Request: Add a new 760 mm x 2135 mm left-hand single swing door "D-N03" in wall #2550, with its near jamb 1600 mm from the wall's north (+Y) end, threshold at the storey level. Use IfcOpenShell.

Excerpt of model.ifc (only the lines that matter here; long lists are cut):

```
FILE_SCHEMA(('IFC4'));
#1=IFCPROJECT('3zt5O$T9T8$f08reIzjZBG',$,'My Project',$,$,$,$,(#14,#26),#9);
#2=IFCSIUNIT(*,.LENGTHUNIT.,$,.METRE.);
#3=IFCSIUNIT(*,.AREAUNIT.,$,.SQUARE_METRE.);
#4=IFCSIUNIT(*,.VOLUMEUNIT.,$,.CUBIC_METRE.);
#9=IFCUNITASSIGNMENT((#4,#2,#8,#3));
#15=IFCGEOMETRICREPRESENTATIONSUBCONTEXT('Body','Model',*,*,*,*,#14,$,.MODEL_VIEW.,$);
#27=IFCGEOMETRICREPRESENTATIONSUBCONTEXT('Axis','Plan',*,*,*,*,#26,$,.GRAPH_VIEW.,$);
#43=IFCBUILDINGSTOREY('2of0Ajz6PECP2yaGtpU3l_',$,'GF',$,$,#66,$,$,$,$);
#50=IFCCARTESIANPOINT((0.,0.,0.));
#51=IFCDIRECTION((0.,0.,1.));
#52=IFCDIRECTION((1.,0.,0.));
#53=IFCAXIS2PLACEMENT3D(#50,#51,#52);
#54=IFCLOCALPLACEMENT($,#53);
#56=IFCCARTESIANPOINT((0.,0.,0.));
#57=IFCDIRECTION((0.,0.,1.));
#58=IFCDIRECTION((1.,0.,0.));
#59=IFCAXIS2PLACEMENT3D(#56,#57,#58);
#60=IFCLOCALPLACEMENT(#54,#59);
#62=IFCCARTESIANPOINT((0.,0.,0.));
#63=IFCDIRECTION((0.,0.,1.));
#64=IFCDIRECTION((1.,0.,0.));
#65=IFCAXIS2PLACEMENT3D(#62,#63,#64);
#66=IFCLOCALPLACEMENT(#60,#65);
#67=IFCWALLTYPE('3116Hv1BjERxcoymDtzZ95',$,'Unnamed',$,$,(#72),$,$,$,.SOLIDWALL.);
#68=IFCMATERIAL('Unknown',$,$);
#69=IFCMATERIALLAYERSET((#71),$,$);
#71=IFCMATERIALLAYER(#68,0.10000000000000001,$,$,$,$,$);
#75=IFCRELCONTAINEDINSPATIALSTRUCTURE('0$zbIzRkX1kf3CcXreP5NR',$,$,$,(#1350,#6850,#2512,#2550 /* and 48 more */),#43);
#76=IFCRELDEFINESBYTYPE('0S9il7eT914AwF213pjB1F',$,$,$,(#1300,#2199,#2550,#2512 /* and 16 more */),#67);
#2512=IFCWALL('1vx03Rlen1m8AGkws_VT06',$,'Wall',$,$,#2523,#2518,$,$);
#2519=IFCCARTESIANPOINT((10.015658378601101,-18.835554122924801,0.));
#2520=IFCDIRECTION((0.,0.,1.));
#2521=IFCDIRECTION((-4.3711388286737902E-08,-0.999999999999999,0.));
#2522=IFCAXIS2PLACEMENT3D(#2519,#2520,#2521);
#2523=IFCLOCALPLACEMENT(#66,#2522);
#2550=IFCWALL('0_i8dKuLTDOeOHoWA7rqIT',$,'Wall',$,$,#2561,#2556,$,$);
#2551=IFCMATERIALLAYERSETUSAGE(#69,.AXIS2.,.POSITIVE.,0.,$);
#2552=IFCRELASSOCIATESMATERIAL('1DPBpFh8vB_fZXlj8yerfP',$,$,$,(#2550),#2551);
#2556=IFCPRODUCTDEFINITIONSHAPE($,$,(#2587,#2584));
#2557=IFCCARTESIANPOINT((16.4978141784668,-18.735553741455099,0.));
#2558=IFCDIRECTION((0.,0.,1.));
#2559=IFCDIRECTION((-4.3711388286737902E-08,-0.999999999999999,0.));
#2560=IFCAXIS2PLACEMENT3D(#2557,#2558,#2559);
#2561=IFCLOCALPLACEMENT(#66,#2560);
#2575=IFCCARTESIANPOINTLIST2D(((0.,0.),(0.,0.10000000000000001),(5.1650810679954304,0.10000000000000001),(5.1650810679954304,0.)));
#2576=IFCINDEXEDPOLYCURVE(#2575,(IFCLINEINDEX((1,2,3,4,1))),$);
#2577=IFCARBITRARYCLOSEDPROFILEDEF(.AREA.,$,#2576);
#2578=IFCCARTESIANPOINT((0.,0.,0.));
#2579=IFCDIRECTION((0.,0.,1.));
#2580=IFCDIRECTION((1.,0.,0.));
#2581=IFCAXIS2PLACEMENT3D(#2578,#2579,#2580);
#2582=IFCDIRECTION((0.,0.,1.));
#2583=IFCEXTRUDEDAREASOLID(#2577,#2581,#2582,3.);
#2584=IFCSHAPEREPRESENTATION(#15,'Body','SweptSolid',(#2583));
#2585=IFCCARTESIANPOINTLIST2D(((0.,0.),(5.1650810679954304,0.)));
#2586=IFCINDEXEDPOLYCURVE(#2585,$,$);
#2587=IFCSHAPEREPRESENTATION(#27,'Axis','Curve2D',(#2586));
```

```python
import numpy as np
import ifcopenshell
import ifcopenshell.api.feature
import ifcopenshell.api.geometry
import ifcopenshell.api.root
import ifcopenshell.api.spatial
import ifcopenshell.geom
import ifcopenshell.util.element
import ifcopenshell.util.placement
import ifcopenshell.util.representation
import ifcopenshell.util.shape
import ifcopenshell.util.unit

model = ifcopenshell.open("model.ifc")
unit_scale = ifcopenshell.util.unit.calculate_unit_scale(model)
settings = ifcopenshell.geom.settings()


def volume(element):
    """Net volume in cubic metres, openings subtracted."""
    shape = ifcopenshell.geom.create_shape(settings, element)
    return ifcopenshell.util.shape.get_volume(shape.geometry)


wall = model.by_guid("0_i8dKuLTDOeOHoWA7rqIT")
storey = ifcopenshell.util.element.get_container(wall, ifc_class="IfcBuildingStorey")
context = ifcopenshell.util.representation.get_context(model, "Model", "Body", "MODEL_VIEW")
before = volume(wall)

width, height, from_end, sill = 0.76, 2.135, 1.6, 0.0  # metres

# The wall runs along its own X axis, and the end named is its -X end.
wall_shape = ifcopenshell.geom.create_shape(settings, wall)
x, y, z = ifcopenshell.util.shape.get_vertices(wall_shape.geometry).T
start = x.min() + from_end
face, thickness = float(y.min()), float(y.max() - y.min())
wall_matrix = ifcopenshell.util.placement.get_local_placement(wall.ObjectPlacement)
level = ifcopenshell.util.placement.get_local_placement(storey.ObjectPlacement)[2, 3]


def in_wall(x, y):
    """Placement at x, y metres in the wall's axes, at sill height."""
    matrix = wall_matrix.copy()
    matrix[:, 3] = wall_matrix @ np.array([x / unit_scale, y / unit_scale, 0.0, 1.0])
    matrix[2, 3] = level + sill / unit_scale
    return matrix


# Opening: a box that overshoots both wall faces by 50 mm.
opening = ifcopenshell.api.root.create_entity(model, ifc_class="IfcOpeningElement", predefined_type="OPENING")
box = ifcopenshell.api.geometry.add_wall_representation(
    model, context=context, length=width, height=height, thickness=thickness + 0.1
)
ifcopenshell.api.geometry.assign_representation(model, product=opening, representation=box)
ifcopenshell.api.geometry.edit_object_placement(model, product=opening, matrix=in_wall(start, face - 0.05), is_si=False)
ifcopenshell.api.feature.add_feature(model, feature=opening, element=wall)

door = ifcopenshell.api.root.create_entity(model, ifc_class="IfcDoor", name="D-N03", predefined_type="DOOR")
door.OverallWidth, door.OverallHeight = width / unit_scale, height / unit_scale
door.OperationType = "SINGLE_SWING_LEFT"
body = ifcopenshell.api.geometry.add_door_representation(
    model,
    context=context,
    overall_width=door.OverallWidth,
    overall_height=door.OverallHeight,
    operation_type="SINGLE_SWING_LEFT",
    lining_properties={"LiningDepth": thickness / unit_scale, "ThresholdDepth": thickness / unit_scale},
)
ifcopenshell.api.geometry.assign_representation(model, product=door, representation=body)
ifcopenshell.api.spatial.assign_container(model, products=[door], relating_structure=storey)
ifcopenshell.api.feature.add_filling(model, opening=opening, element=door)

# The lining spans the wall, so the door starts at the wall face.
ifcopenshell.api.geometry.edit_object_placement(model, product=door, matrix=in_wall(start, face), is_si=False)

after = volume(wall)

print(f"wall volume {before:.3f} -> {after:.3f} m3")

model.write("model_v2.ifc")
```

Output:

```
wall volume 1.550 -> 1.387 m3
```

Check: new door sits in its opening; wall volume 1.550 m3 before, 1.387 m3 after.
